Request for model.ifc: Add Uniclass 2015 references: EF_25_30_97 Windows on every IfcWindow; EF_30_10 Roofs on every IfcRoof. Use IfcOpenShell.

First a look at what the model holds.

```python
import ifcopenshell

model = ifcopenshell.open("model.ifc")
print(model.schema)
print("classifications:", [c.Name for c in model.by_type("IfcClassification")])
for ifc_class in ("IfcDoor", "IfcRoof", "IfcStair", "IfcWall", "IfcWindow"):
    print(ifc_class, len(model.by_type(ifc_class)))
```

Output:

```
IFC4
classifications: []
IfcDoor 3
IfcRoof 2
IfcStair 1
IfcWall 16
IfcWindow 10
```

```python
import ifcopenshell
import ifcopenshell.api.classification

model = ifcopenshell.open("model.ifc")

system = ifcopenshell.api.classification.add_classification(model, classification="Uniclass 2015")

codes = {
    "IfcWindow": ("EF_25_30_97", "Windows"),
    "IfcRoof": ("EF_30_10", "Roofs"),
}
for ifc_class, (code, name) in codes.items():
    products = model.by_type(ifc_class)
    ifcopenshell.api.classification.add_reference(
        model, products=products, classification=system, identification=code, name=name
    )
    print(code, len(products))

model.write("model-out.ifc")
```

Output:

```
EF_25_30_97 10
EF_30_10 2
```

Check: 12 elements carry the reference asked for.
